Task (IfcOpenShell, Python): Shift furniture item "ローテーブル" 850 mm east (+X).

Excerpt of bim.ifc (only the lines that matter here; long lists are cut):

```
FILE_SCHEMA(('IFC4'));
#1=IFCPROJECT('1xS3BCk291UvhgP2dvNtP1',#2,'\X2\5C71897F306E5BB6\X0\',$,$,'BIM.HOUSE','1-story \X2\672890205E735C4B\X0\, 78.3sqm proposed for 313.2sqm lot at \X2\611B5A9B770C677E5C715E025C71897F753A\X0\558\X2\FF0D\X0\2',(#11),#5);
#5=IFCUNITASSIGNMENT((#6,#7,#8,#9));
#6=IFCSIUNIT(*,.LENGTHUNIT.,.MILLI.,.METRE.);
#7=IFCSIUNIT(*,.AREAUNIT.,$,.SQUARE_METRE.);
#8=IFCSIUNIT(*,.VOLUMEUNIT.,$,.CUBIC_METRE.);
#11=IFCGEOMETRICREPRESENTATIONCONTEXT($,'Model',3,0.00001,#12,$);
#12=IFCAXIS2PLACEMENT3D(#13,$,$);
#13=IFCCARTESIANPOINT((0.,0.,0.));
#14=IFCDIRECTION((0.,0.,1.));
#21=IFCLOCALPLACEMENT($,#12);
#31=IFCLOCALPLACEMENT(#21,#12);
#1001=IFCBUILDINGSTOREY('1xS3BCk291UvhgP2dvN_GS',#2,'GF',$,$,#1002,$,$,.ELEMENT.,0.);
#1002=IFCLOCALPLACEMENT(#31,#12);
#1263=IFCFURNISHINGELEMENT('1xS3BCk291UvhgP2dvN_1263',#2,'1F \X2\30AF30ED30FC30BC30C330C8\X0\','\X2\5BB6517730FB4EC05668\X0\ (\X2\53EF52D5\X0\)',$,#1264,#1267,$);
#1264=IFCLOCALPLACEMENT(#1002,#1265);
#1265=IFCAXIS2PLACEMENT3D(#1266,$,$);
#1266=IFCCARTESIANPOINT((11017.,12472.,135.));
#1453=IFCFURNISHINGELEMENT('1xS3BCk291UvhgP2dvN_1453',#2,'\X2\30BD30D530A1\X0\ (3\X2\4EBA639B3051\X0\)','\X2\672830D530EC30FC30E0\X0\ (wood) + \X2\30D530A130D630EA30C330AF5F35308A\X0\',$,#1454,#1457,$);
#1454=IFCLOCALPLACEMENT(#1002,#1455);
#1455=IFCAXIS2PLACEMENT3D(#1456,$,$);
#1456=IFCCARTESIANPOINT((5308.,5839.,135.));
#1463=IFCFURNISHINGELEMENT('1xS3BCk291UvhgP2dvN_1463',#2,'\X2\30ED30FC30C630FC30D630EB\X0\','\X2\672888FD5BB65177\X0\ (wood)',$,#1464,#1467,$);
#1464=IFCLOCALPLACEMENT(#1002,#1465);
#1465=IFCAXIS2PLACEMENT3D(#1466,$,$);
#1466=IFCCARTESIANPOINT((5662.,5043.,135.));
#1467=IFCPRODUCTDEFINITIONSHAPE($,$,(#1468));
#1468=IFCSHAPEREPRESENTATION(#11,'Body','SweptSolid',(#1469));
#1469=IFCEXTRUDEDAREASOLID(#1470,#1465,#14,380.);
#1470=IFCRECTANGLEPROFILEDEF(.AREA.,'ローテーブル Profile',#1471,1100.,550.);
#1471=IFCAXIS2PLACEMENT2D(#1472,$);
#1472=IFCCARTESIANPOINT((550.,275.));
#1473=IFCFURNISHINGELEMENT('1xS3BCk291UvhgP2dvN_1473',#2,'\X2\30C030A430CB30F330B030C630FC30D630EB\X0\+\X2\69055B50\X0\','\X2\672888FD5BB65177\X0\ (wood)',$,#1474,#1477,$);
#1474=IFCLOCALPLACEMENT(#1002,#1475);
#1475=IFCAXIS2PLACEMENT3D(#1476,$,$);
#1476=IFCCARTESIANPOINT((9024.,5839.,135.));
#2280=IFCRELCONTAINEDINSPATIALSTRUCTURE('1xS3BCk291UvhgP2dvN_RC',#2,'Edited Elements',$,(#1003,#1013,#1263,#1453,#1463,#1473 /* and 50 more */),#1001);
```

```python
import ifcopenshell
import ifcopenshell.api.geometry
import ifcopenshell.util.placement

model = ifcopenshell.open("bim.ifc")

item = model.by_guid("1xS3BCk291UvhgP2dvN_1463")
matrix = ifcopenshell.util.placement.get_local_placement(item.ObjectPlacement)
matrix[0, 3] += 850.0
ifcopenshell.api.geometry.edit_object_placement(model, product=item, matrix=matrix, is_si=False)

print(ifcopenshell.util.placement.get_local_placement(item.ObjectPlacement).round(3) + 0.0)

model.write("bim_rev.ifc")
```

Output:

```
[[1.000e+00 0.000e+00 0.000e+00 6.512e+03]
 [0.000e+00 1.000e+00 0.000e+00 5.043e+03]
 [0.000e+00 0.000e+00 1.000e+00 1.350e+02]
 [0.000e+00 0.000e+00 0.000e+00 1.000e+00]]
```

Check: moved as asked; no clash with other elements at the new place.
